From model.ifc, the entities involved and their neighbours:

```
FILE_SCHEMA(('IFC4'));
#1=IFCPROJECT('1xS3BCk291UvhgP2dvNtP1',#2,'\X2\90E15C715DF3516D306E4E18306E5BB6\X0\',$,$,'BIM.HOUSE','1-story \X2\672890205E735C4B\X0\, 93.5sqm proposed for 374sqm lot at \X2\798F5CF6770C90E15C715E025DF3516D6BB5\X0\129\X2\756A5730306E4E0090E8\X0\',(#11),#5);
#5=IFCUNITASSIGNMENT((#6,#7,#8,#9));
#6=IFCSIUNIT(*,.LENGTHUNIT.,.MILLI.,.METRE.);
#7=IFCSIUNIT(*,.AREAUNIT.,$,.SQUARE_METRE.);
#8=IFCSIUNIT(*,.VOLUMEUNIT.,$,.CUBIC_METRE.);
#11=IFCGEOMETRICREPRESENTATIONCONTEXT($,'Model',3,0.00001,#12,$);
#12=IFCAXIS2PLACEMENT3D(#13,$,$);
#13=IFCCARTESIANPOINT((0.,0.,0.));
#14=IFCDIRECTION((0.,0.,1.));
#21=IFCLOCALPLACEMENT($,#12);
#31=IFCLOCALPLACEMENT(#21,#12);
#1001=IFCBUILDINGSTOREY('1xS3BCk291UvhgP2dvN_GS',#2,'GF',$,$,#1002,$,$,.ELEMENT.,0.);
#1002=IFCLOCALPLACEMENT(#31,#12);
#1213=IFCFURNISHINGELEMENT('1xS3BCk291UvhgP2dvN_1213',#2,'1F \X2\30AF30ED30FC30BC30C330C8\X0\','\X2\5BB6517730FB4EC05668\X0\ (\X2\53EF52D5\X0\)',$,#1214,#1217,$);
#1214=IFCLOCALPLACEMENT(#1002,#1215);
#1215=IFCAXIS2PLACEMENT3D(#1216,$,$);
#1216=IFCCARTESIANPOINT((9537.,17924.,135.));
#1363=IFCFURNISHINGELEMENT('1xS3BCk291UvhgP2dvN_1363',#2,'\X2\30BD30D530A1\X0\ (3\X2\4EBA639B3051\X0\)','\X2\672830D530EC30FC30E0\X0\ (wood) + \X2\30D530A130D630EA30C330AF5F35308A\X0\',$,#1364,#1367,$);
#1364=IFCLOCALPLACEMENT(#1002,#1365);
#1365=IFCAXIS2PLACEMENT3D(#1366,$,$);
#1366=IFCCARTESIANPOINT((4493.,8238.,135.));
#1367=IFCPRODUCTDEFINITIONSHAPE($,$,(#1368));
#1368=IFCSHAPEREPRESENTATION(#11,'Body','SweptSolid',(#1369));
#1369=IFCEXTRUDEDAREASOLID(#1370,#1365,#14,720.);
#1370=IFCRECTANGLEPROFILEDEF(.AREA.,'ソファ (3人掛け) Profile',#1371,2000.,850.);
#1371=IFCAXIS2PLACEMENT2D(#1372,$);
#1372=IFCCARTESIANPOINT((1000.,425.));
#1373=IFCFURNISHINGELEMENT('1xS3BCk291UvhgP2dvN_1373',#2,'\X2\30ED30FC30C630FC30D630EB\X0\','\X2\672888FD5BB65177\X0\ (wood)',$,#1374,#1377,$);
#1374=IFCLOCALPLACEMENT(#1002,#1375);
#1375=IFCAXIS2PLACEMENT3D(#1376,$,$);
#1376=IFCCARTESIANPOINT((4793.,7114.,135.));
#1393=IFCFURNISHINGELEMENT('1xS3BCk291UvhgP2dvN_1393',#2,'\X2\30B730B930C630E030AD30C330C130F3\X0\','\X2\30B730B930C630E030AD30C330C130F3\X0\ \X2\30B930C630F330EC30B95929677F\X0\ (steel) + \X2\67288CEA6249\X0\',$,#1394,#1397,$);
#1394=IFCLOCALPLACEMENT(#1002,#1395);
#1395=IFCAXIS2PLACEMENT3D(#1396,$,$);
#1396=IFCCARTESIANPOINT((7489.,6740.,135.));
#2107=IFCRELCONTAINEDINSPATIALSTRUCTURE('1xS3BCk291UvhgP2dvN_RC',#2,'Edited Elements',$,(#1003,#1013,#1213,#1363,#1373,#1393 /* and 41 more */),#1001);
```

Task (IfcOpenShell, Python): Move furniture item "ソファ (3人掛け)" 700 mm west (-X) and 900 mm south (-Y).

```python
import ifcopenshell
import ifcopenshell.api.geometry
import ifcopenshell.util.placement

model = ifcopenshell.open("model.ifc")

item = model.by_id(1363)
matrix = ifcopenshell.util.placement.get_local_placement(item.ObjectPlacement)
matrix[0, 3] -= 700.0
matrix[1, 3] -= 900.0
ifcopenshell.api.geometry.edit_object_placement(model, product=item, matrix=matrix, is_si=False)

print(ifcopenshell.util.placement.get_local_placement(item.ObjectPlacement).round(3) + 0.0)

model.write("model-out.ifc")
```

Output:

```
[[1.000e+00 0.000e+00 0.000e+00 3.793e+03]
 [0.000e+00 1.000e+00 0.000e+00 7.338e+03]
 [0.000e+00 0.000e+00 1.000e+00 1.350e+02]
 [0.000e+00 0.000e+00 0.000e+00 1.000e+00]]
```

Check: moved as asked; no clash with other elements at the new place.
